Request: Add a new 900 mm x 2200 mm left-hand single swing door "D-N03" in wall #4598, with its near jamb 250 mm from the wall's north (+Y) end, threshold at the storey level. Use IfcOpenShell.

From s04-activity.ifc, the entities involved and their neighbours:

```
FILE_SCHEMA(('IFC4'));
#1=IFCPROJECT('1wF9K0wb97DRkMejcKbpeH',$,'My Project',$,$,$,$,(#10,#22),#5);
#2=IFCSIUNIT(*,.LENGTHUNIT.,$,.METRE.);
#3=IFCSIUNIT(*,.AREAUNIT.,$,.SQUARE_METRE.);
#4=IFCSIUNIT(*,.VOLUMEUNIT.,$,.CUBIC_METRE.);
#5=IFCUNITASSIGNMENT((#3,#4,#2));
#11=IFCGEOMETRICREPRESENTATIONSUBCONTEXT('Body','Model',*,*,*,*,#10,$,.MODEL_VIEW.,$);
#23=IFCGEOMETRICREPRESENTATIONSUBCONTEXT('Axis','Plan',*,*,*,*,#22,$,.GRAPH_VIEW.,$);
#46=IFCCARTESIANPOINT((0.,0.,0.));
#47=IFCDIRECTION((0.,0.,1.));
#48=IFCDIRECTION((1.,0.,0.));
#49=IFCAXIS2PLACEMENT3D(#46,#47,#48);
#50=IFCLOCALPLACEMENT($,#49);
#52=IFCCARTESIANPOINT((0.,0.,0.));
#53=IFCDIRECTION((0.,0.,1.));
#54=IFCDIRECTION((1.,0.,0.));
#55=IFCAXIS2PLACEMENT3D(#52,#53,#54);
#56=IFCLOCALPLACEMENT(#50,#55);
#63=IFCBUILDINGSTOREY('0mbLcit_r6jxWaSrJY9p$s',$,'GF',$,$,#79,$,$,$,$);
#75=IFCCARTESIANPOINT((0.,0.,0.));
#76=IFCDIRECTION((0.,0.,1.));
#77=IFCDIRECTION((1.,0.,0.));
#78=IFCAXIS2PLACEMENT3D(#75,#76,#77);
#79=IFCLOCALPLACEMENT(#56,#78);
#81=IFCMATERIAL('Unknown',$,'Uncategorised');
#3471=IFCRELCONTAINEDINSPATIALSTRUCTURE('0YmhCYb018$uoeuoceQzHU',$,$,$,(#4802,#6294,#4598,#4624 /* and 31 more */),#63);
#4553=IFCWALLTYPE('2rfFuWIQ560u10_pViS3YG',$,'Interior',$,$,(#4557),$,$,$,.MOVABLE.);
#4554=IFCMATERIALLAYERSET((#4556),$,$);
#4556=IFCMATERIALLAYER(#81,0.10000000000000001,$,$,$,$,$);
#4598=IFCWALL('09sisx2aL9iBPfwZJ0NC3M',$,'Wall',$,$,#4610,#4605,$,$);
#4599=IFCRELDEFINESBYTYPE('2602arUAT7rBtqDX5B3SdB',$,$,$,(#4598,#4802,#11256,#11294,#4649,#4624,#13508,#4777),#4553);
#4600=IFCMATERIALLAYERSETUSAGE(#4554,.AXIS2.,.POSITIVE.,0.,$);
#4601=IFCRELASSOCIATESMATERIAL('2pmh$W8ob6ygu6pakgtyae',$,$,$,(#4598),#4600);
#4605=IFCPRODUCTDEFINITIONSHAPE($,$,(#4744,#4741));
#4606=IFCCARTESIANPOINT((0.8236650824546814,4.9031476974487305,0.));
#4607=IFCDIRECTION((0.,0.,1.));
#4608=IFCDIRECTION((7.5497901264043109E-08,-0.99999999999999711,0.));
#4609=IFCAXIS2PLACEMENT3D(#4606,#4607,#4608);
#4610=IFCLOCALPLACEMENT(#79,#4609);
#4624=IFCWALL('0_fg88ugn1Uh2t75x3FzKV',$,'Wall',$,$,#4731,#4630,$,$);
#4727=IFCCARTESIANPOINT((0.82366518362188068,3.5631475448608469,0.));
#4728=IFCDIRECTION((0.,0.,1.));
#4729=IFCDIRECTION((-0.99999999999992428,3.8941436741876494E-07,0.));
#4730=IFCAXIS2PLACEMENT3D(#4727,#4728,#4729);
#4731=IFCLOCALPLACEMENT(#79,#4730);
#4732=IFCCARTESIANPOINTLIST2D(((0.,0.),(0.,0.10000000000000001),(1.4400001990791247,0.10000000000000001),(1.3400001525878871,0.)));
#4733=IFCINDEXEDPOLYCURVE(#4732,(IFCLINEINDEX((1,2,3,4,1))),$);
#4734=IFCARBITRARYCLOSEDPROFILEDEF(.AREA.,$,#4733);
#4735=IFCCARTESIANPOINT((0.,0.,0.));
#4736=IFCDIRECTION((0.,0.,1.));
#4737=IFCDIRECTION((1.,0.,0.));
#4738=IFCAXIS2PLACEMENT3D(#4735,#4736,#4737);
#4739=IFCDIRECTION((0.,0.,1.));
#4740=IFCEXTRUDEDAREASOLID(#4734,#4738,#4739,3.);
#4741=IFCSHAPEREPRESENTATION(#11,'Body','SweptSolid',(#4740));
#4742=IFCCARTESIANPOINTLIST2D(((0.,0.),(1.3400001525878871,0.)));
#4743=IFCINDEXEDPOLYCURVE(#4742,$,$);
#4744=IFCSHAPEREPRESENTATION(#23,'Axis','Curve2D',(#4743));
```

```python
import numpy as np
import ifcopenshell
import ifcopenshell.api.feature
import ifcopenshell.api.geometry
import ifcopenshell.api.root
import ifcopenshell.api.spatial
import ifcopenshell.geom
import ifcopenshell.util.element
import ifcopenshell.util.placement
import ifcopenshell.util.representation
import ifcopenshell.util.shape
import ifcopenshell.util.unit

model = ifcopenshell.open("s04-activity.ifc")
unit_scale = ifcopenshell.util.unit.calculate_unit_scale(model)
settings = ifcopenshell.geom.settings()


def volume(element):
    """Net volume in cubic metres, openings subtracted."""
    shape = ifcopenshell.geom.create_shape(settings, element)
    return ifcopenshell.util.shape.get_volume(shape.geometry)


wall = model.by_guid("09sisx2aL9iBPfwZJ0NC3M")
storey = ifcopenshell.util.element.get_container(wall, ifc_class="IfcBuildingStorey")
context = ifcopenshell.util.representation.get_context(model, "Model", "Body", "MODEL_VIEW")
before = volume(wall)

width, height, from_end, sill = 0.9, 2.2, 0.25, 0.0  # metres

# The wall runs along its own X axis, and the end named is its -X end.
wall_shape = ifcopenshell.geom.create_shape(settings, wall)
x, y, z = ifcopenshell.util.shape.get_vertices(wall_shape.geometry).T
start = x.min() + from_end
face, thickness = float(y.min()), float(y.max() - y.min())
wall_matrix = ifcopenshell.util.placement.get_local_placement(wall.ObjectPlacement)
level = ifcopenshell.util.placement.get_local_placement(storey.ObjectPlacement)[2, 3]


def in_wall(x, y):
    """Placement at x, y metres in the wall's axes, at sill height."""
    matrix = wall_matrix.copy()
    matrix[:, 3] = wall_matrix @ np.array([x / unit_scale, y / unit_scale, 0.0, 1.0])
    matrix[2, 3] = level + sill / unit_scale
    return matrix


# Opening: a box that overshoots both wall faces by 50 mm.
opening = ifcopenshell.api.root.create_entity(model, ifc_class="IfcOpeningElement", predefined_type="OPENING")
box = ifcopenshell.api.geometry.add_wall_representation(
    model, context=context, length=width, height=height, thickness=thickness + 0.1
)
ifcopenshell.api.geometry.assign_representation(model, product=opening, representation=box)
ifcopenshell.api.geometry.edit_object_placement(model, product=opening, matrix=in_wall(start, face - 0.05), is_si=False)
ifcopenshell.api.feature.add_feature(model, feature=opening, element=wall)

door = ifcopenshell.api.root.create_entity(model, ifc_class="IfcDoor", name="D-N03", predefined_type="DOOR")
door.OverallWidth, door.OverallHeight = width / unit_scale, height / unit_scale
door.OperationType = "SINGLE_SWING_LEFT"
body = ifcopenshell.api.geometry.add_door_representation(
    model,
    context=context,
    overall_width=door.OverallWidth,
    overall_height=door.OverallHeight,
    operation_type="SINGLE_SWING_LEFT",
    lining_properties={"LiningDepth": thickness / unit_scale, "ThresholdDepth": thickness / unit_scale},
)
ifcopenshell.api.geometry.assign_representation(model, product=door, representation=body)
ifcopenshell.api.spatial.assign_container(model, products=[door], relating_structure=storey)
ifcopenshell.api.feature.add_filling(model, opening=opening, element=door)

# The lining spans the wall, so the door starts at the wall face.
ifcopenshell.api.geometry.edit_object_placement(model, product=door, matrix=in_wall(start, face), is_si=False)

after = volume(wall)

print(f"wall volume {before:.3f} -> {after:.3f} m3")

model.write("s04-activity_v2.ifc")
```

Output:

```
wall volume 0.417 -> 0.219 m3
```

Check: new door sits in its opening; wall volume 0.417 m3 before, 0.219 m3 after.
